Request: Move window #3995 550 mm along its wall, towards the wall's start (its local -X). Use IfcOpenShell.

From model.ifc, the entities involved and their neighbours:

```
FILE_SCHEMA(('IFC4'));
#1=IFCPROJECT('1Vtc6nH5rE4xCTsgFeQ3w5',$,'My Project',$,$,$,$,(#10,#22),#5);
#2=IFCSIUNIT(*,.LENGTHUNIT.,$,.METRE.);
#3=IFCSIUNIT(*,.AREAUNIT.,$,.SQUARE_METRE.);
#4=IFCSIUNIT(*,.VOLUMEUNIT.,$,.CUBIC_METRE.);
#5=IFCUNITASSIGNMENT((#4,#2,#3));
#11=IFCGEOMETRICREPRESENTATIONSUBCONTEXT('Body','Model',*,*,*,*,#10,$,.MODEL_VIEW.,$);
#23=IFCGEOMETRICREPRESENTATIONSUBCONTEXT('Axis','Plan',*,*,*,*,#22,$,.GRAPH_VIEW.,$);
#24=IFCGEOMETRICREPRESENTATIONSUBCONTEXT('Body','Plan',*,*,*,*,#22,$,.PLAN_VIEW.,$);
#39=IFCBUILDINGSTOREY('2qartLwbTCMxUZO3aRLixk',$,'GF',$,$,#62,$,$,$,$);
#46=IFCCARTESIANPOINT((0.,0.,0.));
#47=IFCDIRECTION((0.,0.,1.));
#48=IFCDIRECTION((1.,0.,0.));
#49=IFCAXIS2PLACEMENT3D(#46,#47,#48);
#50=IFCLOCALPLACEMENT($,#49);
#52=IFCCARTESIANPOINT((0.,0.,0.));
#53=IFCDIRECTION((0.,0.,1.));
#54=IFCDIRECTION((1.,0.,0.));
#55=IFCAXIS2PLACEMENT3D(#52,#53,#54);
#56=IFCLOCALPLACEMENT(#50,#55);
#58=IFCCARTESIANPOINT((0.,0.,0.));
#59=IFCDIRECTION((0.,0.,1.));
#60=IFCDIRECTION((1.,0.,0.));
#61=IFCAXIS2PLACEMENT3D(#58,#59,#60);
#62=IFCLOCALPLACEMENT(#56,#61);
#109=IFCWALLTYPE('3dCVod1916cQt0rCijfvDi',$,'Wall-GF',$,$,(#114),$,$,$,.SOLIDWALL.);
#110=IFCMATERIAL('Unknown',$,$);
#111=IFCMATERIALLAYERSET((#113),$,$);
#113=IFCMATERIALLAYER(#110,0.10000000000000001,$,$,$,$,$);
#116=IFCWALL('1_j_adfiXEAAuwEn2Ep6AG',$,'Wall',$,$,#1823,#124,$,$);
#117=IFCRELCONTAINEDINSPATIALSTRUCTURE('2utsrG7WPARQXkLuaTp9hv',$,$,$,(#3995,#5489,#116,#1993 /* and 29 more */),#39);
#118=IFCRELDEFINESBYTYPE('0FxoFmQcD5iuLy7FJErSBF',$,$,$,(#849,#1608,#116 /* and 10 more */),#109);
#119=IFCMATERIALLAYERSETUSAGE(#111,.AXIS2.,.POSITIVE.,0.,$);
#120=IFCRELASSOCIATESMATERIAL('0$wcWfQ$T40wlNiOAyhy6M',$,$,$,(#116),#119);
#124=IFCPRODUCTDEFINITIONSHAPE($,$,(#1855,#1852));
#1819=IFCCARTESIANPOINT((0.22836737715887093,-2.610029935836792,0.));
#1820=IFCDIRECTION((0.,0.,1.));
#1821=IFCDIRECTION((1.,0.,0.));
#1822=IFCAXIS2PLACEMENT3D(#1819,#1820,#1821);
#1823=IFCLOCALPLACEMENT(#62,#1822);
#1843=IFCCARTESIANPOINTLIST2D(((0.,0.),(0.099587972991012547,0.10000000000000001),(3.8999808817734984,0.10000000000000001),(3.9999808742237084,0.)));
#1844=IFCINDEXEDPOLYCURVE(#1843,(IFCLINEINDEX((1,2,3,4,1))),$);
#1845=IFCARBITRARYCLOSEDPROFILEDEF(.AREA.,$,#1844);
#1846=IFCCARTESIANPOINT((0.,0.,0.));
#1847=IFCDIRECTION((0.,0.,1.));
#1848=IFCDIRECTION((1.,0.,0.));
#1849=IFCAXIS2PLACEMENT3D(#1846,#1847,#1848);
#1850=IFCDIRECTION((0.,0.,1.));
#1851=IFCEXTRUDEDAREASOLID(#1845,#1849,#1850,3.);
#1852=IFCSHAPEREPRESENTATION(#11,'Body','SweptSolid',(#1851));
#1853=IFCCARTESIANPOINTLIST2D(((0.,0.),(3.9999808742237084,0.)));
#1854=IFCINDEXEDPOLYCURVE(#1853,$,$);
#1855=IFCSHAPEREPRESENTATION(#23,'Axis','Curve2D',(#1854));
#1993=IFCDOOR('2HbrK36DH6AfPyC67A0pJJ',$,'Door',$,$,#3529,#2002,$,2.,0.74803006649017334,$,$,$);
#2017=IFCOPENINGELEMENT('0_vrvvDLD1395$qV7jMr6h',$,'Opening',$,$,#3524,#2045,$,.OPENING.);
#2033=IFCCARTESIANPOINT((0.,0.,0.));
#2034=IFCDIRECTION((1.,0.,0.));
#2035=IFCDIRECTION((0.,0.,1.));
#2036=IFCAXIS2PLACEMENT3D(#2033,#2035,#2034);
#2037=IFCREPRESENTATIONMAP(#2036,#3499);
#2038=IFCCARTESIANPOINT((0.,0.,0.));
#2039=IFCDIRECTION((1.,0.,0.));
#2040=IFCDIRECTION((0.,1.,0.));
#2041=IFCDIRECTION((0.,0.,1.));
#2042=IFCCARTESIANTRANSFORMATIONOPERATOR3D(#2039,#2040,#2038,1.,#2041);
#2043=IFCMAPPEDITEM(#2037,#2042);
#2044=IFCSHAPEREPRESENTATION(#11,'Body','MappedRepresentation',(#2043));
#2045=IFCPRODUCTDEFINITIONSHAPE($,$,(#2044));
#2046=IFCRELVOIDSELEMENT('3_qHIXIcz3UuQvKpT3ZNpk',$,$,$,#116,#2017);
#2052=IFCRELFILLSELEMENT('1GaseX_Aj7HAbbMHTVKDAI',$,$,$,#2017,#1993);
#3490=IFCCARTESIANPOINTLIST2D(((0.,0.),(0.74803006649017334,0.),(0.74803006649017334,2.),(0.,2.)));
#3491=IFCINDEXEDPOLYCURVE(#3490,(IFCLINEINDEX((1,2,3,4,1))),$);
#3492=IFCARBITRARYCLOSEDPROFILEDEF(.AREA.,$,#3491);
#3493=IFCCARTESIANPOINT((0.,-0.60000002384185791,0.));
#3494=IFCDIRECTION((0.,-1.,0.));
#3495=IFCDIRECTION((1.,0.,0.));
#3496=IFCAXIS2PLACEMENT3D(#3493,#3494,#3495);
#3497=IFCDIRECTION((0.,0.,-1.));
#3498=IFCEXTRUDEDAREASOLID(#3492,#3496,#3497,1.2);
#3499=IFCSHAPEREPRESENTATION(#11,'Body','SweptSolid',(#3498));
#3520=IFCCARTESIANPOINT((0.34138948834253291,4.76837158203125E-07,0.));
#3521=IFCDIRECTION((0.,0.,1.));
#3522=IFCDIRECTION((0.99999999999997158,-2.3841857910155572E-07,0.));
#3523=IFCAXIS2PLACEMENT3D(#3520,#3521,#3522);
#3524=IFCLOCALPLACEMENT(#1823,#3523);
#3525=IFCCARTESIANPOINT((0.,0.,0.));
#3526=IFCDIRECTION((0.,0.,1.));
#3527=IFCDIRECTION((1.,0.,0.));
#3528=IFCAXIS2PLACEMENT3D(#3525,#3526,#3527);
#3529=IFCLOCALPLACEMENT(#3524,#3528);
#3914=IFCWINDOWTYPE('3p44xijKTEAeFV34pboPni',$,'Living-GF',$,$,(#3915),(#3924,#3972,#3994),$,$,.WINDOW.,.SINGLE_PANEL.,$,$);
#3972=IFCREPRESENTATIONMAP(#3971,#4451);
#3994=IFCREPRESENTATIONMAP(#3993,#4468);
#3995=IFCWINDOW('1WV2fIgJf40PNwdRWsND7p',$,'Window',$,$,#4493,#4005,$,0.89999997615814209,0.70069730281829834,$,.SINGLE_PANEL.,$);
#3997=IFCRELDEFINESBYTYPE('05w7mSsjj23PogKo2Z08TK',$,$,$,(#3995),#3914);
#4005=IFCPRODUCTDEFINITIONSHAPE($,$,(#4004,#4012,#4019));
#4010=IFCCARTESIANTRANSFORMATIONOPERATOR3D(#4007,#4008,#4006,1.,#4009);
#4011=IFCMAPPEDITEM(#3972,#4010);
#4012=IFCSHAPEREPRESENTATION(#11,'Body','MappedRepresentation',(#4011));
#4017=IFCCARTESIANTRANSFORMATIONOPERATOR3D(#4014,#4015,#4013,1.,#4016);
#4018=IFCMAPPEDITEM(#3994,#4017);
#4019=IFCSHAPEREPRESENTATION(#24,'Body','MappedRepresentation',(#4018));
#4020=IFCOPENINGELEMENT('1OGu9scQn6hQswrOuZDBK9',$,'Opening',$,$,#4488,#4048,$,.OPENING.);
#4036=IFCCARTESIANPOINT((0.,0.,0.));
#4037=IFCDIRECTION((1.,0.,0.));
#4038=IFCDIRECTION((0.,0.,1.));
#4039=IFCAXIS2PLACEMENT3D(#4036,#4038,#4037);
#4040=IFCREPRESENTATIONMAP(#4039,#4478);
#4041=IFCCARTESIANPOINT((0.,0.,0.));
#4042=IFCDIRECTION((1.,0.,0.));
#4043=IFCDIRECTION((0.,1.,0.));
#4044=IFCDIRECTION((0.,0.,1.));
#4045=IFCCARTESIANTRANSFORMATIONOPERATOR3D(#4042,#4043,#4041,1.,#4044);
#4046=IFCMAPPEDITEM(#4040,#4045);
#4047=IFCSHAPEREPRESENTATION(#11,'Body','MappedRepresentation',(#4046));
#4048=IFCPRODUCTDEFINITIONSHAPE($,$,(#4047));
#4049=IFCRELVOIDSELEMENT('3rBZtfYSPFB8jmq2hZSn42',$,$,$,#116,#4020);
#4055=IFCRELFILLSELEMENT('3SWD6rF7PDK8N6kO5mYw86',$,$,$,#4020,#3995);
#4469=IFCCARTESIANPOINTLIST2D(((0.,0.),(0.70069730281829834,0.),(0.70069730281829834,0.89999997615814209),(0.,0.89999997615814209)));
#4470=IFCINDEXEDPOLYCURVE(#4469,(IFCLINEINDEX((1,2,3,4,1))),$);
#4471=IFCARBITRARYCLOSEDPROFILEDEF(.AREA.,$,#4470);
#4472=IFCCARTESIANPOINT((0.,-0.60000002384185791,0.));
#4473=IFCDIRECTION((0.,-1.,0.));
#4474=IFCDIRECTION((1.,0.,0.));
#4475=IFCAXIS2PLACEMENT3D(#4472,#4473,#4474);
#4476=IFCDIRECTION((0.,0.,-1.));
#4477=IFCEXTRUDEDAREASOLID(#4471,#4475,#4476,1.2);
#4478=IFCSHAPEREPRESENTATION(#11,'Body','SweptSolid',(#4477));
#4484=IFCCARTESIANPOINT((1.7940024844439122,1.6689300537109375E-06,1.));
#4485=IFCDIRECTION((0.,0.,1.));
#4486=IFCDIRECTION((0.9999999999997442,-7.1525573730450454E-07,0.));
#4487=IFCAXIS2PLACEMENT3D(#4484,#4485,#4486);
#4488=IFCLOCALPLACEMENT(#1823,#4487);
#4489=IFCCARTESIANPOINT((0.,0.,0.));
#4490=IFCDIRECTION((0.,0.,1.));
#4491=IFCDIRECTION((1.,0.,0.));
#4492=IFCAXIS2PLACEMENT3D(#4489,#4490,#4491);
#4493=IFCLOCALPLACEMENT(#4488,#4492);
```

```python
import ifcopenshell
import ifcopenshell.api.geometry
import ifcopenshell.util.placement
import ifcopenshell.util.unit

model = ifcopenshell.open("model.ifc")
unit_scale = ifcopenshell.util.unit.calculate_unit_scale(model)

window = model.by_guid("1WV2fIgJf40PNwdRWsND7p")
opening = window.FillsVoids[0].RelatingOpeningElement
wall = opening.VoidsElements[0].RelatingBuildingElement

wall_matrix = ifcopenshell.util.placement.get_local_placement(wall.ObjectPlacement)
shift = wall_matrix[:3, 0] * -0.55 / unit_scale
before = ifcopenshell.util.placement.get_local_placement(window.ObjectPlacement)[:3, 3].copy()

# The window is placed relative to its opening, so it follows when the opening moves.
matrix = ifcopenshell.util.placement.get_local_placement(opening.ObjectPlacement)
matrix[:3, 3] += shift
ifcopenshell.api.geometry.edit_object_placement(
    model, product=opening, matrix=matrix, is_si=False, should_transform_children=True
)

after = ifcopenshell.util.placement.get_local_placement(window.ObjectPlacement)[:3, 3]
print("window moved by", (after - before).round(3) + 0.0)

model.write("model_edited.ifc")
```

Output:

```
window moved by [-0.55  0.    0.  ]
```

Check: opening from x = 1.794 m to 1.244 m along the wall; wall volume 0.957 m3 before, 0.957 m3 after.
